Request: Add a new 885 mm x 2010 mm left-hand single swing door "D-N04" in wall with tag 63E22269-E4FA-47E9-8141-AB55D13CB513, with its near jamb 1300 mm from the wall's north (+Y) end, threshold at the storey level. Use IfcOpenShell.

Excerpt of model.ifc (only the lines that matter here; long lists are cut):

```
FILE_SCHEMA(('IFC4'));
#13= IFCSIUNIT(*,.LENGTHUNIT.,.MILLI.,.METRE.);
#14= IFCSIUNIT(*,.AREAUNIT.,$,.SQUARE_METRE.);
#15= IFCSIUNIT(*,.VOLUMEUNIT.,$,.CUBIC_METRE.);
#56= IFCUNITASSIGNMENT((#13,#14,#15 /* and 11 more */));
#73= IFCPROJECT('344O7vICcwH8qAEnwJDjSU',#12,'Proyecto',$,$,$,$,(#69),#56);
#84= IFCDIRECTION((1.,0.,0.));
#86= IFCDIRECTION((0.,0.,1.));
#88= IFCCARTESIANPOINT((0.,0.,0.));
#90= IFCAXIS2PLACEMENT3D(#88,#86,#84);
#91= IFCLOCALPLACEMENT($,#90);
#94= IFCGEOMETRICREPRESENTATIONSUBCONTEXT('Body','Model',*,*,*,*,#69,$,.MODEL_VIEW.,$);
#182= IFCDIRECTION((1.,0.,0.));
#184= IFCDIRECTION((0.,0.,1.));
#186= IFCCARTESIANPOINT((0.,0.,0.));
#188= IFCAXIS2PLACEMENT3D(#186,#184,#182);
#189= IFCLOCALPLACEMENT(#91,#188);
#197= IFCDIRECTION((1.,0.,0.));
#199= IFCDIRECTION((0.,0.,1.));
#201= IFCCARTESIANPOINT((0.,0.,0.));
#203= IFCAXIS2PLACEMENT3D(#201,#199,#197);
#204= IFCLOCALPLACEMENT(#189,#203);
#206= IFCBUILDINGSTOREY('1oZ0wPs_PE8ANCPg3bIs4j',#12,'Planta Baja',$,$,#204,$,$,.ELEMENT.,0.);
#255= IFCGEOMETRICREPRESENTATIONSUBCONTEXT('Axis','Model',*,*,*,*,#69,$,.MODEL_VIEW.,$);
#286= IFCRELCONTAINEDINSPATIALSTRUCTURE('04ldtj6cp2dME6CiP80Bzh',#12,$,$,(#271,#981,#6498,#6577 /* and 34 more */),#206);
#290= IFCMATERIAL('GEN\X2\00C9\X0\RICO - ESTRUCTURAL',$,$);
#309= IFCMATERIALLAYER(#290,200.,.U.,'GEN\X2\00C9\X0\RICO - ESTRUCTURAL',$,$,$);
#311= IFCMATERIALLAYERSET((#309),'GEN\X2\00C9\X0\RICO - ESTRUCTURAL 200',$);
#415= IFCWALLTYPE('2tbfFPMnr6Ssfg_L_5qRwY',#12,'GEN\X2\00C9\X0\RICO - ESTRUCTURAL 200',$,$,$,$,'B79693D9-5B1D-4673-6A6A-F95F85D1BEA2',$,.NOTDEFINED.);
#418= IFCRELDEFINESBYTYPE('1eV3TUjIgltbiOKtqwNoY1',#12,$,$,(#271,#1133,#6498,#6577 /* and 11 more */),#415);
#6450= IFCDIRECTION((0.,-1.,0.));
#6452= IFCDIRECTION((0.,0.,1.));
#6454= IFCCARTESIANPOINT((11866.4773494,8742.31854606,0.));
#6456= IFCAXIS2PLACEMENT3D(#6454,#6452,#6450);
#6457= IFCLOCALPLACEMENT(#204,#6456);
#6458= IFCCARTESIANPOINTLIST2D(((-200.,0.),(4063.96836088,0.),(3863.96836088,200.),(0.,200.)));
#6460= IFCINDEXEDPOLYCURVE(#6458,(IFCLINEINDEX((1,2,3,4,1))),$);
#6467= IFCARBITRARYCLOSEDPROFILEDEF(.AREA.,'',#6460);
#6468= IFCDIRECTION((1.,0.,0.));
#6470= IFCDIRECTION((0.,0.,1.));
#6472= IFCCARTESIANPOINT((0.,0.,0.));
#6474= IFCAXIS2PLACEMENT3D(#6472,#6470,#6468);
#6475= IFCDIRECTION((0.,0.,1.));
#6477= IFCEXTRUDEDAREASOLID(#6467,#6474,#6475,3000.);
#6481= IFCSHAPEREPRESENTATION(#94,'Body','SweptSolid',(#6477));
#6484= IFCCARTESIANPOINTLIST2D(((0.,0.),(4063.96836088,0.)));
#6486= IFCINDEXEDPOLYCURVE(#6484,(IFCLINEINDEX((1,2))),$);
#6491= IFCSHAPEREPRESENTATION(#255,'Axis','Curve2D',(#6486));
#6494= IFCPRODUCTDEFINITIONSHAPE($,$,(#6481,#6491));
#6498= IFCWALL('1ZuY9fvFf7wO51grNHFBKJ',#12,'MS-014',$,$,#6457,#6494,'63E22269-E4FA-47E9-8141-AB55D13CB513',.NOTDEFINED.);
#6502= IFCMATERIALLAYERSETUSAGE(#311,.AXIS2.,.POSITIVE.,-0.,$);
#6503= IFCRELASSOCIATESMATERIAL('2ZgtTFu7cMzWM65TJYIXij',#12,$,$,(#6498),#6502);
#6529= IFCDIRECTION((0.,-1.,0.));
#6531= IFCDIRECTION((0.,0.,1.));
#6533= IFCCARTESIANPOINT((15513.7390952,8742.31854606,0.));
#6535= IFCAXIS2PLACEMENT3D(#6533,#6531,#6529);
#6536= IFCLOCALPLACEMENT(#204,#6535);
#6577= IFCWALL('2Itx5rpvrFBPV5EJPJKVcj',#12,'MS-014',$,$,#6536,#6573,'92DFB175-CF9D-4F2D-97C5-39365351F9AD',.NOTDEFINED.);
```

```python
import numpy as np
import ifcopenshell
import ifcopenshell.api.feature
import ifcopenshell.api.geometry
import ifcopenshell.api.root
import ifcopenshell.api.spatial
import ifcopenshell.geom
import ifcopenshell.util.element
import ifcopenshell.util.placement
import ifcopenshell.util.representation
import ifcopenshell.util.shape
import ifcopenshell.util.unit

model = ifcopenshell.open("model.ifc")
unit_scale = ifcopenshell.util.unit.calculate_unit_scale(model)
settings = ifcopenshell.geom.settings()


def volume(element):
    """Net volume in cubic metres, openings subtracted."""
    shape = ifcopenshell.geom.create_shape(settings, element)
    return ifcopenshell.util.shape.get_volume(shape.geometry)


wall = model.by_guid("1ZuY9fvFf7wO51grNHFBKJ")
storey = ifcopenshell.util.element.get_container(wall, ifc_class="IfcBuildingStorey")
context = ifcopenshell.util.representation.get_context(model, "Model", "Body", "MODEL_VIEW")
before = volume(wall)

width, height, from_end, sill = 0.885, 2.01, 1.3, 0.0  # metres

# The wall runs along its own X axis, and the end named is its -X end.
wall_shape = ifcopenshell.geom.create_shape(settings, wall)
x, y, z = ifcopenshell.util.shape.get_vertices(wall_shape.geometry).T
start = x.min() + from_end
face, thickness = float(y.min()), float(y.max() - y.min())
wall_matrix = ifcopenshell.util.placement.get_local_placement(wall.ObjectPlacement)
level = ifcopenshell.util.placement.get_local_placement(storey.ObjectPlacement)[2, 3]


def in_wall(x, y):
    """Placement at x, y metres in the wall's axes, at sill height."""
    matrix = wall_matrix.copy()
    matrix[:, 3] = wall_matrix @ np.array([x / unit_scale, y / unit_scale, 0.0, 1.0])
    matrix[2, 3] = level + sill / unit_scale
    return matrix


# Opening: a box that overshoots both wall faces by 50 mm.
opening = ifcopenshell.api.root.create_entity(model, ifc_class="IfcOpeningElement", predefined_type="OPENING")
box = ifcopenshell.api.geometry.add_wall_representation(
    model, context=context, length=width, height=height, thickness=thickness + 0.1
)
ifcopenshell.api.geometry.assign_representation(model, product=opening, representation=box)
ifcopenshell.api.geometry.edit_object_placement(model, product=opening, matrix=in_wall(start, face - 0.05), is_si=False)
ifcopenshell.api.feature.add_feature(model, feature=opening, element=wall)

door = ifcopenshell.api.root.create_entity(model, ifc_class="IfcDoor", name="D-N04", predefined_type="DOOR")
door.OverallWidth, door.OverallHeight = width / unit_scale, height / unit_scale
door.OperationType = "SINGLE_SWING_LEFT"
body = ifcopenshell.api.geometry.add_door_representation(
    model,
    context=context,
    overall_width=door.OverallWidth,
    overall_height=door.OverallHeight,
    operation_type="SINGLE_SWING_LEFT",
    lining_properties={"LiningDepth": thickness / unit_scale, "ThresholdDepth": thickness / unit_scale},
)
ifcopenshell.api.geometry.assign_representation(model, product=door, representation=body)
ifcopenshell.api.spatial.assign_container(model, products=[door], relating_structure=storey)
ifcopenshell.api.feature.add_filling(model, opening=opening, element=door)

# The lining spans the wall, so the door starts at the wall face.
ifcopenshell.api.geometry.edit_object_placement(model, product=door, matrix=in_wall(start, face), is_si=False)

after = volume(wall)

print(f"wall volume {before:.3f} -> {after:.3f} m3")

model.write("model_v2.ifc")
```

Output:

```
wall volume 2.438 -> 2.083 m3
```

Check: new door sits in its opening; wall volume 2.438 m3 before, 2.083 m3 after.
